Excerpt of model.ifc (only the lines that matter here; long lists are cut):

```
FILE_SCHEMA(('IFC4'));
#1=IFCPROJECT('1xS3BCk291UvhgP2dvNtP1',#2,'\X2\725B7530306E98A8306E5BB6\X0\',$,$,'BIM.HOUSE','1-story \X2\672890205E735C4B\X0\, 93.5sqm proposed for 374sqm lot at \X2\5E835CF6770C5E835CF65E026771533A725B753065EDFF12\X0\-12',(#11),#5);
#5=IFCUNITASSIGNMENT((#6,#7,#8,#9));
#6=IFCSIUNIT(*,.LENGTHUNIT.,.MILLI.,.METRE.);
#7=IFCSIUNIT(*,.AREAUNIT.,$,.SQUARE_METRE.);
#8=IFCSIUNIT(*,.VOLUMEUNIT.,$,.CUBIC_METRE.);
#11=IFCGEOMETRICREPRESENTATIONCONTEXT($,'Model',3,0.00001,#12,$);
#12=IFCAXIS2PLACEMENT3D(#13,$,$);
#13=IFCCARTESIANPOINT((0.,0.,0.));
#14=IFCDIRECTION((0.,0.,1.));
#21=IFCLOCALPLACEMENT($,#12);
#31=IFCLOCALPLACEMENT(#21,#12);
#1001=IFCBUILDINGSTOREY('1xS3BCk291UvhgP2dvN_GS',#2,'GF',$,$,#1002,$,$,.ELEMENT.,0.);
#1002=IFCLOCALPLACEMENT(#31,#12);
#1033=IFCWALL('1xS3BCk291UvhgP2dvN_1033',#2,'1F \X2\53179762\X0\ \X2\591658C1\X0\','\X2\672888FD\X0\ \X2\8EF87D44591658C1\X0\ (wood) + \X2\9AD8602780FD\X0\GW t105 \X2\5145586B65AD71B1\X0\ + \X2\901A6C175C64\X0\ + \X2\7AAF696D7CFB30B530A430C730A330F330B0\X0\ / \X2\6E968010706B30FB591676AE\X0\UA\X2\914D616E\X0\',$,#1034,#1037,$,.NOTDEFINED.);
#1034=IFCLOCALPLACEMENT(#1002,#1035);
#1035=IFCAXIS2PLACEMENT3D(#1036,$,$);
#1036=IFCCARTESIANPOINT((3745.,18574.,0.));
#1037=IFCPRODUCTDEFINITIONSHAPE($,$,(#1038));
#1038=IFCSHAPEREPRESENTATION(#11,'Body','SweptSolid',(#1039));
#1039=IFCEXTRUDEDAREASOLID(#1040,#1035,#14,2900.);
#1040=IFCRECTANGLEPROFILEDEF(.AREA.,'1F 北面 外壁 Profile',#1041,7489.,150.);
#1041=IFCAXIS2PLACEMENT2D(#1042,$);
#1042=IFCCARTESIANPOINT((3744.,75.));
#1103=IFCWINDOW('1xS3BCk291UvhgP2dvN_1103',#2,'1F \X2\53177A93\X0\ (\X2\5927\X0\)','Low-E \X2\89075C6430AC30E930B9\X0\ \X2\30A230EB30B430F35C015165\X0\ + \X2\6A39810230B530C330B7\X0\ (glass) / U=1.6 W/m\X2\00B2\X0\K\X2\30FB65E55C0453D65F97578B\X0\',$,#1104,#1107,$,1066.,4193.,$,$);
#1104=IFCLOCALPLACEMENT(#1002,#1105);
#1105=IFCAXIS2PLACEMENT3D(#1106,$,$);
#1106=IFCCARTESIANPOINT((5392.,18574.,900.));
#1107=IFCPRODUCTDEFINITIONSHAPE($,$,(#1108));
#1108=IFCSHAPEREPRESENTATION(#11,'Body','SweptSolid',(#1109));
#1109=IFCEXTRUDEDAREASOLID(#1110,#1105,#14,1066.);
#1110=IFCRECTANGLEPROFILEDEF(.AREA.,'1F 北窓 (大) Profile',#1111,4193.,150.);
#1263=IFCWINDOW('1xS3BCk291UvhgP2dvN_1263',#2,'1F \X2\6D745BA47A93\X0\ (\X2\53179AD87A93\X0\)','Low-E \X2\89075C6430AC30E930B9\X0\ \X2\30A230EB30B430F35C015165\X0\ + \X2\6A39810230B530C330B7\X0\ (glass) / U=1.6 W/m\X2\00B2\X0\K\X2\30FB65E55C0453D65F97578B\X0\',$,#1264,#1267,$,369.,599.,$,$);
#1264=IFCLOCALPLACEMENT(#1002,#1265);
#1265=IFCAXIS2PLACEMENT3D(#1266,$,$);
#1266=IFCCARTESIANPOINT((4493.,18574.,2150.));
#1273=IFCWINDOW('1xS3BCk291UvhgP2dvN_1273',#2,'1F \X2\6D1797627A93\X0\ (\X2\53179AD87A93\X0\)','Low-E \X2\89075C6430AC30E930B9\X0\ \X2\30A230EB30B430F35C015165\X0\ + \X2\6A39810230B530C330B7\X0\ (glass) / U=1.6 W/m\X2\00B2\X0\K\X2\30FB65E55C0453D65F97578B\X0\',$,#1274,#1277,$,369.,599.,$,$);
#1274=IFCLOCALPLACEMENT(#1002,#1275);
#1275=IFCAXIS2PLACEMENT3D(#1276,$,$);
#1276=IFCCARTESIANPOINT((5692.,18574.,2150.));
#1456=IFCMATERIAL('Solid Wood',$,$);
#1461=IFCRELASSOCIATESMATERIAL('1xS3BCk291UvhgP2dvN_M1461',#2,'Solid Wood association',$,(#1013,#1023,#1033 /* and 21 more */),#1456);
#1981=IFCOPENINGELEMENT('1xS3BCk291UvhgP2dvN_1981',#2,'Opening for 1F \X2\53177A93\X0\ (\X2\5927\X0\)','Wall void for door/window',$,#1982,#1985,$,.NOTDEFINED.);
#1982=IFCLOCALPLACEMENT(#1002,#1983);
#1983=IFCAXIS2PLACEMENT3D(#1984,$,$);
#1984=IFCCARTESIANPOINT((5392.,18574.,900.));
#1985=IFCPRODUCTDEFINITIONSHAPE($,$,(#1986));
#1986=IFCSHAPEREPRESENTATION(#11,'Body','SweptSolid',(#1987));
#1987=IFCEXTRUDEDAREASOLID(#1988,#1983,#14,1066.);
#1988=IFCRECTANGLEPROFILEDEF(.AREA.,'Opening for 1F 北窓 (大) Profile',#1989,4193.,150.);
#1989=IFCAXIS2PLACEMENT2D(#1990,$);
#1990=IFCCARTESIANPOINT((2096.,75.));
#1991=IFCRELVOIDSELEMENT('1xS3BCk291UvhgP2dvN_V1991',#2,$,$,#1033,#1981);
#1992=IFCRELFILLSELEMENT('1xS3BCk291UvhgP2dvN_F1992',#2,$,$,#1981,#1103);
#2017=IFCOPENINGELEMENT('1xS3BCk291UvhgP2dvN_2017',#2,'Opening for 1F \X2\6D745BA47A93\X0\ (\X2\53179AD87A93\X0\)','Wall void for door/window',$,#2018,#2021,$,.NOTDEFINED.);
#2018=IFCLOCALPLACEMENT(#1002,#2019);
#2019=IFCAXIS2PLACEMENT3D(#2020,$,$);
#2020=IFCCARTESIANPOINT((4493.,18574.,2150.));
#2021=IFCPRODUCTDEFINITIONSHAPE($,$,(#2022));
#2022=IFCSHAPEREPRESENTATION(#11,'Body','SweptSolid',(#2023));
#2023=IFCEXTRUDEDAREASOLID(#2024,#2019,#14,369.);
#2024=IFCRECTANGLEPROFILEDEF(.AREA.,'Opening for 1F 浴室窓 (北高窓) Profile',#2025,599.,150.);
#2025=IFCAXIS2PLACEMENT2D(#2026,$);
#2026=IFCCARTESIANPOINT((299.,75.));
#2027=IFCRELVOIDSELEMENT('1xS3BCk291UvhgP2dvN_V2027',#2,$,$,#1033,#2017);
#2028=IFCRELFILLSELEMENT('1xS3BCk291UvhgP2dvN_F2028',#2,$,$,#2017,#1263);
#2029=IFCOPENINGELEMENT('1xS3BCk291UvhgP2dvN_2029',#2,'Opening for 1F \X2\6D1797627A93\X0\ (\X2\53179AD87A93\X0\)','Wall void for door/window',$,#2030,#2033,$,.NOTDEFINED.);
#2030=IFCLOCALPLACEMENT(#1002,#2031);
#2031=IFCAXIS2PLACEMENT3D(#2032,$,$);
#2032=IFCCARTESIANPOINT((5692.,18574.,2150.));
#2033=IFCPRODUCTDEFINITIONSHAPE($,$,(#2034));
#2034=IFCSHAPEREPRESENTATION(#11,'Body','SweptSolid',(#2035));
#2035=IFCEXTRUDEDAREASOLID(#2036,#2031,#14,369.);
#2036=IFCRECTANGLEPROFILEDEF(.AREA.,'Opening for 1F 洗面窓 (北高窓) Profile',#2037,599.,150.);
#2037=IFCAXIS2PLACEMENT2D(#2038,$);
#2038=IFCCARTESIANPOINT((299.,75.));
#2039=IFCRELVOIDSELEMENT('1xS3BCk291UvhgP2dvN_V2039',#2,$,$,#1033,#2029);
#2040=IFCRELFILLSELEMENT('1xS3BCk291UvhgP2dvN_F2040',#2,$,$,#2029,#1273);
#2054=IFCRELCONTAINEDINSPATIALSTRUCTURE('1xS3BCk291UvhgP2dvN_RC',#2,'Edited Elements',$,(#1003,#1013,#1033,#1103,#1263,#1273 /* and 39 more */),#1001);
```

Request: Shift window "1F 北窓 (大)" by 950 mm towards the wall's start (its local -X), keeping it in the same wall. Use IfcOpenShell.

```python
import ifcopenshell
import ifcopenshell.api.geometry
import ifcopenshell.util.placement
import ifcopenshell.util.unit

model = ifcopenshell.open("model.ifc")
unit_scale = ifcopenshell.util.unit.calculate_unit_scale(model)

window = model.by_guid("1xS3BCk291UvhgP2dvN_1103")
opening = window.FillsVoids[0].RelatingOpeningElement
wall = opening.VoidsElements[0].RelatingBuildingElement

wall_matrix = ifcopenshell.util.placement.get_local_placement(wall.ObjectPlacement)
shift = wall_matrix[:3, 0] * -0.95 / unit_scale
before = ifcopenshell.util.placement.get_local_placement(window.ObjectPlacement)[:3, 3].copy()

# The window is not placed relative to its opening, so move both.
for product in (opening, window):
    matrix = ifcopenshell.util.placement.get_local_placement(product.ObjectPlacement)
    matrix[:3, 3] += shift
    ifcopenshell.api.geometry.edit_object_placement(model, product=product, matrix=matrix, is_si=False)

after = ifcopenshell.util.placement.get_local_placement(window.ObjectPlacement)[:3, 3]
print("window moved by", (after - before).round(3) + 0.0)

model.write("model_updated.ifc")
```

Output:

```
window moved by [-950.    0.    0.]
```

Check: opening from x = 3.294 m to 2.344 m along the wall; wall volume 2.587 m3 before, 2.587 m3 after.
